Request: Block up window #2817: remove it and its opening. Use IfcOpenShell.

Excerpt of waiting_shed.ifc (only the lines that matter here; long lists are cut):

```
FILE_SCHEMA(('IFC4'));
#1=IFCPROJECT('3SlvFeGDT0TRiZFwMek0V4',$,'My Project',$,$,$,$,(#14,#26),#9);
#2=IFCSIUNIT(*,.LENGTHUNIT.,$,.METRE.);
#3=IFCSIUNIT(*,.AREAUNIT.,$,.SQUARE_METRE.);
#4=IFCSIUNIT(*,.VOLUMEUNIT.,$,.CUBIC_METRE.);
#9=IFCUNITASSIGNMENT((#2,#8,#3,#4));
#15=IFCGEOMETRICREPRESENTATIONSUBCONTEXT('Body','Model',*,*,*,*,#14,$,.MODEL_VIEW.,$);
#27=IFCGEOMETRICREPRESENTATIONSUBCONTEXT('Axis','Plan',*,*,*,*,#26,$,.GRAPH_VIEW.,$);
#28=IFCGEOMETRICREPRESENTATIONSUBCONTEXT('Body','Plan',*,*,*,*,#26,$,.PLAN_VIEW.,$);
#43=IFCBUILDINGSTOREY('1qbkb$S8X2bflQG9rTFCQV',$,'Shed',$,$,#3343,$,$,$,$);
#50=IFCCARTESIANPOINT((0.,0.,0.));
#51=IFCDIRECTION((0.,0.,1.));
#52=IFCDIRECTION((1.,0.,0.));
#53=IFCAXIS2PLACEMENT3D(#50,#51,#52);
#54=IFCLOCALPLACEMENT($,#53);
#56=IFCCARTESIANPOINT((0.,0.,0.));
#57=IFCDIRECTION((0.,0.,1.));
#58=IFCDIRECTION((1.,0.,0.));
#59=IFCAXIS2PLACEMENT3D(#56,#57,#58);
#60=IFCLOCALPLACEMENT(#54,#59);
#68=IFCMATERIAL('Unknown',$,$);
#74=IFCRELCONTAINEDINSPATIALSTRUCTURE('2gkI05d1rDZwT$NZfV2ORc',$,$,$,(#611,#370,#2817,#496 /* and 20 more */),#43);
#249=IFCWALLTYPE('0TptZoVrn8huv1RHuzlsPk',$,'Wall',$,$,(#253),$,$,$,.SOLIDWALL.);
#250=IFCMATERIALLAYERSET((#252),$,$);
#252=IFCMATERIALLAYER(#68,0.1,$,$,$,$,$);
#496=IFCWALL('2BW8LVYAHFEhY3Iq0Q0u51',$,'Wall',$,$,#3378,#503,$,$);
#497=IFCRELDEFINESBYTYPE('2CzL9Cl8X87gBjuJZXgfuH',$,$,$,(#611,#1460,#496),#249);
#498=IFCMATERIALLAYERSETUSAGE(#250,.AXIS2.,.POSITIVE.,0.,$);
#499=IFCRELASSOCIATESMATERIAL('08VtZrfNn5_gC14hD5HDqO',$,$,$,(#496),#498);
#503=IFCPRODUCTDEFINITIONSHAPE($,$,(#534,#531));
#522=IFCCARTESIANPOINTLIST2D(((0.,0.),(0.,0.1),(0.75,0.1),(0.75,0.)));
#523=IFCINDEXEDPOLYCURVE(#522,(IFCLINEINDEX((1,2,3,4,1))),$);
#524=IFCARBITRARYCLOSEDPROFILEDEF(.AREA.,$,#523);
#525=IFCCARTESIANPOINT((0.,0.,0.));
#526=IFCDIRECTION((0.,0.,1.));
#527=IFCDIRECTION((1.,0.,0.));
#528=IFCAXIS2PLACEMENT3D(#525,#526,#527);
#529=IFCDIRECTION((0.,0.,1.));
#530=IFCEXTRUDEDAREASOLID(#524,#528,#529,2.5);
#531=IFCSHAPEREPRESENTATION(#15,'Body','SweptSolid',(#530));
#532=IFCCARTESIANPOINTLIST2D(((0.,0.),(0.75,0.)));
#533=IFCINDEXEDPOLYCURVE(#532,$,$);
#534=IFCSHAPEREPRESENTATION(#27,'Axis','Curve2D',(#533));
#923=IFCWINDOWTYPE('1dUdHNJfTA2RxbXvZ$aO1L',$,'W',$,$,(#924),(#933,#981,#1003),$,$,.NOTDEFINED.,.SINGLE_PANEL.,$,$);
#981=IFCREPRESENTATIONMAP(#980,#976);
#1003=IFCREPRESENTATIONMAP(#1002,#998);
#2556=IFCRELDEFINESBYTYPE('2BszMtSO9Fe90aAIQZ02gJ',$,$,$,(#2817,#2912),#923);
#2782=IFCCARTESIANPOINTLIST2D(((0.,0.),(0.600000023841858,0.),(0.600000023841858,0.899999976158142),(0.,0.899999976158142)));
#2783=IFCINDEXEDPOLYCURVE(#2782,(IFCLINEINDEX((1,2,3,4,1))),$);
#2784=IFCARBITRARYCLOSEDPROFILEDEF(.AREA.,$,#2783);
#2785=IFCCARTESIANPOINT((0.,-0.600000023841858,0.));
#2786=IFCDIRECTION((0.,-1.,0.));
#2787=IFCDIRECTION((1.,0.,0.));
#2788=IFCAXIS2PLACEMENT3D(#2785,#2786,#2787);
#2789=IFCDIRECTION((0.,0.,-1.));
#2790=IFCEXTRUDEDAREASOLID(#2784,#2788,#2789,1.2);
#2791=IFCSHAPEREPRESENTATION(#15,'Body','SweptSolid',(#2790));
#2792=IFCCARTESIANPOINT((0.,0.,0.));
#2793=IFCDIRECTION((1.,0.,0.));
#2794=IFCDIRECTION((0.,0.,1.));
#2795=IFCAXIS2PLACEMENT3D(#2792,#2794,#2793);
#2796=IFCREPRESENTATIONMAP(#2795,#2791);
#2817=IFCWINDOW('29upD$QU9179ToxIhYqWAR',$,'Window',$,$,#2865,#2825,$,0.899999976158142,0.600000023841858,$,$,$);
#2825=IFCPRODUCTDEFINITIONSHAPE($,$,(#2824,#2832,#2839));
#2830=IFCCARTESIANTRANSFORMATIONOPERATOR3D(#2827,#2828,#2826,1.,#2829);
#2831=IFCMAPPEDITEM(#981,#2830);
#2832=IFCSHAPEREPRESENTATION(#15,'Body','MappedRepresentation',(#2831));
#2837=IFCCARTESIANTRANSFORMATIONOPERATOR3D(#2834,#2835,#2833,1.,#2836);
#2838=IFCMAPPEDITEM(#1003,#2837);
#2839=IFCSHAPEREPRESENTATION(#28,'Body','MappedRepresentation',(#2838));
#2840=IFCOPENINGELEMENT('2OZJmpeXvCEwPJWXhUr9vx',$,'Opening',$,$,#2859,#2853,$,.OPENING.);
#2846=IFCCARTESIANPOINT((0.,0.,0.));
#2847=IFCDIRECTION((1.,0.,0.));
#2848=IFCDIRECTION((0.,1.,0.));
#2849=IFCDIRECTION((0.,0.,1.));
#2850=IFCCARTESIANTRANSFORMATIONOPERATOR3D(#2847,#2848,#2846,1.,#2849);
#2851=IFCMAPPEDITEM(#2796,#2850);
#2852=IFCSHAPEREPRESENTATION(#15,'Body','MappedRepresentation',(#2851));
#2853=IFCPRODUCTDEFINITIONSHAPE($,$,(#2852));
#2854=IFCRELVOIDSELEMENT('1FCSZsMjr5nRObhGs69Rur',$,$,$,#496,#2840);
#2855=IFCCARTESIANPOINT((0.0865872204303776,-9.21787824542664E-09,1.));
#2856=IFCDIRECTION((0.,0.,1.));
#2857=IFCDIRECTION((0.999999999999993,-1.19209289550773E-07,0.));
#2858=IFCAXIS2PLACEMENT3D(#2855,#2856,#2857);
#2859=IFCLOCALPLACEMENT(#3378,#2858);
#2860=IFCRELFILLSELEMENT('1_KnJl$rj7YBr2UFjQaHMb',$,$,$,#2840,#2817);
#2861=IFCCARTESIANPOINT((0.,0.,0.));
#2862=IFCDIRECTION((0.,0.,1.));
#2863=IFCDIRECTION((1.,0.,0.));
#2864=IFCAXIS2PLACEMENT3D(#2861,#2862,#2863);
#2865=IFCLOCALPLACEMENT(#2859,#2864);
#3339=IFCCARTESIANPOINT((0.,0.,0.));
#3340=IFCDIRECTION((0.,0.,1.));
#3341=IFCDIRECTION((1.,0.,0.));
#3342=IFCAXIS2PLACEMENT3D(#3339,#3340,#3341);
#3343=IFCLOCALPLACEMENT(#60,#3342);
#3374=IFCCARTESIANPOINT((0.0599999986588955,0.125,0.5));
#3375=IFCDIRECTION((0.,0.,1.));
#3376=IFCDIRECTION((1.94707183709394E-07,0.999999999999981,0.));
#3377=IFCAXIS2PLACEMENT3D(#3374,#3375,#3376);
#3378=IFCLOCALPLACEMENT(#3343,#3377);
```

```python
import ifcopenshell
import ifcopenshell.api.feature
import ifcopenshell.api.root
import ifcopenshell.geom
import ifcopenshell.util.shape

model = ifcopenshell.open("waiting_shed.ifc")
settings = ifcopenshell.geom.settings()


def volume(element):
    """Net volume in cubic metres, openings subtracted."""
    shape = ifcopenshell.geom.create_shape(settings, element)
    return ifcopenshell.util.shape.get_volume(shape.geometry)


window = model.by_guid("29upD$QU9179ToxIhYqWAR")
opening = window.FillsVoids[0].RelatingOpeningElement
wall = opening.VoidsElements[0].RelatingBuildingElement
before = volume(wall)

ifcopenshell.api.root.remove_product(model, product=window)
ifcopenshell.api.feature.remove_feature(model, feature=opening)

after = volume(wall)

print(f"wall volume {before:.3f} -> {after:.3f} m3")

model.write("waiting_shed_v2.ifc")
```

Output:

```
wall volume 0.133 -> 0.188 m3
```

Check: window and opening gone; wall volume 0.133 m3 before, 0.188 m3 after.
